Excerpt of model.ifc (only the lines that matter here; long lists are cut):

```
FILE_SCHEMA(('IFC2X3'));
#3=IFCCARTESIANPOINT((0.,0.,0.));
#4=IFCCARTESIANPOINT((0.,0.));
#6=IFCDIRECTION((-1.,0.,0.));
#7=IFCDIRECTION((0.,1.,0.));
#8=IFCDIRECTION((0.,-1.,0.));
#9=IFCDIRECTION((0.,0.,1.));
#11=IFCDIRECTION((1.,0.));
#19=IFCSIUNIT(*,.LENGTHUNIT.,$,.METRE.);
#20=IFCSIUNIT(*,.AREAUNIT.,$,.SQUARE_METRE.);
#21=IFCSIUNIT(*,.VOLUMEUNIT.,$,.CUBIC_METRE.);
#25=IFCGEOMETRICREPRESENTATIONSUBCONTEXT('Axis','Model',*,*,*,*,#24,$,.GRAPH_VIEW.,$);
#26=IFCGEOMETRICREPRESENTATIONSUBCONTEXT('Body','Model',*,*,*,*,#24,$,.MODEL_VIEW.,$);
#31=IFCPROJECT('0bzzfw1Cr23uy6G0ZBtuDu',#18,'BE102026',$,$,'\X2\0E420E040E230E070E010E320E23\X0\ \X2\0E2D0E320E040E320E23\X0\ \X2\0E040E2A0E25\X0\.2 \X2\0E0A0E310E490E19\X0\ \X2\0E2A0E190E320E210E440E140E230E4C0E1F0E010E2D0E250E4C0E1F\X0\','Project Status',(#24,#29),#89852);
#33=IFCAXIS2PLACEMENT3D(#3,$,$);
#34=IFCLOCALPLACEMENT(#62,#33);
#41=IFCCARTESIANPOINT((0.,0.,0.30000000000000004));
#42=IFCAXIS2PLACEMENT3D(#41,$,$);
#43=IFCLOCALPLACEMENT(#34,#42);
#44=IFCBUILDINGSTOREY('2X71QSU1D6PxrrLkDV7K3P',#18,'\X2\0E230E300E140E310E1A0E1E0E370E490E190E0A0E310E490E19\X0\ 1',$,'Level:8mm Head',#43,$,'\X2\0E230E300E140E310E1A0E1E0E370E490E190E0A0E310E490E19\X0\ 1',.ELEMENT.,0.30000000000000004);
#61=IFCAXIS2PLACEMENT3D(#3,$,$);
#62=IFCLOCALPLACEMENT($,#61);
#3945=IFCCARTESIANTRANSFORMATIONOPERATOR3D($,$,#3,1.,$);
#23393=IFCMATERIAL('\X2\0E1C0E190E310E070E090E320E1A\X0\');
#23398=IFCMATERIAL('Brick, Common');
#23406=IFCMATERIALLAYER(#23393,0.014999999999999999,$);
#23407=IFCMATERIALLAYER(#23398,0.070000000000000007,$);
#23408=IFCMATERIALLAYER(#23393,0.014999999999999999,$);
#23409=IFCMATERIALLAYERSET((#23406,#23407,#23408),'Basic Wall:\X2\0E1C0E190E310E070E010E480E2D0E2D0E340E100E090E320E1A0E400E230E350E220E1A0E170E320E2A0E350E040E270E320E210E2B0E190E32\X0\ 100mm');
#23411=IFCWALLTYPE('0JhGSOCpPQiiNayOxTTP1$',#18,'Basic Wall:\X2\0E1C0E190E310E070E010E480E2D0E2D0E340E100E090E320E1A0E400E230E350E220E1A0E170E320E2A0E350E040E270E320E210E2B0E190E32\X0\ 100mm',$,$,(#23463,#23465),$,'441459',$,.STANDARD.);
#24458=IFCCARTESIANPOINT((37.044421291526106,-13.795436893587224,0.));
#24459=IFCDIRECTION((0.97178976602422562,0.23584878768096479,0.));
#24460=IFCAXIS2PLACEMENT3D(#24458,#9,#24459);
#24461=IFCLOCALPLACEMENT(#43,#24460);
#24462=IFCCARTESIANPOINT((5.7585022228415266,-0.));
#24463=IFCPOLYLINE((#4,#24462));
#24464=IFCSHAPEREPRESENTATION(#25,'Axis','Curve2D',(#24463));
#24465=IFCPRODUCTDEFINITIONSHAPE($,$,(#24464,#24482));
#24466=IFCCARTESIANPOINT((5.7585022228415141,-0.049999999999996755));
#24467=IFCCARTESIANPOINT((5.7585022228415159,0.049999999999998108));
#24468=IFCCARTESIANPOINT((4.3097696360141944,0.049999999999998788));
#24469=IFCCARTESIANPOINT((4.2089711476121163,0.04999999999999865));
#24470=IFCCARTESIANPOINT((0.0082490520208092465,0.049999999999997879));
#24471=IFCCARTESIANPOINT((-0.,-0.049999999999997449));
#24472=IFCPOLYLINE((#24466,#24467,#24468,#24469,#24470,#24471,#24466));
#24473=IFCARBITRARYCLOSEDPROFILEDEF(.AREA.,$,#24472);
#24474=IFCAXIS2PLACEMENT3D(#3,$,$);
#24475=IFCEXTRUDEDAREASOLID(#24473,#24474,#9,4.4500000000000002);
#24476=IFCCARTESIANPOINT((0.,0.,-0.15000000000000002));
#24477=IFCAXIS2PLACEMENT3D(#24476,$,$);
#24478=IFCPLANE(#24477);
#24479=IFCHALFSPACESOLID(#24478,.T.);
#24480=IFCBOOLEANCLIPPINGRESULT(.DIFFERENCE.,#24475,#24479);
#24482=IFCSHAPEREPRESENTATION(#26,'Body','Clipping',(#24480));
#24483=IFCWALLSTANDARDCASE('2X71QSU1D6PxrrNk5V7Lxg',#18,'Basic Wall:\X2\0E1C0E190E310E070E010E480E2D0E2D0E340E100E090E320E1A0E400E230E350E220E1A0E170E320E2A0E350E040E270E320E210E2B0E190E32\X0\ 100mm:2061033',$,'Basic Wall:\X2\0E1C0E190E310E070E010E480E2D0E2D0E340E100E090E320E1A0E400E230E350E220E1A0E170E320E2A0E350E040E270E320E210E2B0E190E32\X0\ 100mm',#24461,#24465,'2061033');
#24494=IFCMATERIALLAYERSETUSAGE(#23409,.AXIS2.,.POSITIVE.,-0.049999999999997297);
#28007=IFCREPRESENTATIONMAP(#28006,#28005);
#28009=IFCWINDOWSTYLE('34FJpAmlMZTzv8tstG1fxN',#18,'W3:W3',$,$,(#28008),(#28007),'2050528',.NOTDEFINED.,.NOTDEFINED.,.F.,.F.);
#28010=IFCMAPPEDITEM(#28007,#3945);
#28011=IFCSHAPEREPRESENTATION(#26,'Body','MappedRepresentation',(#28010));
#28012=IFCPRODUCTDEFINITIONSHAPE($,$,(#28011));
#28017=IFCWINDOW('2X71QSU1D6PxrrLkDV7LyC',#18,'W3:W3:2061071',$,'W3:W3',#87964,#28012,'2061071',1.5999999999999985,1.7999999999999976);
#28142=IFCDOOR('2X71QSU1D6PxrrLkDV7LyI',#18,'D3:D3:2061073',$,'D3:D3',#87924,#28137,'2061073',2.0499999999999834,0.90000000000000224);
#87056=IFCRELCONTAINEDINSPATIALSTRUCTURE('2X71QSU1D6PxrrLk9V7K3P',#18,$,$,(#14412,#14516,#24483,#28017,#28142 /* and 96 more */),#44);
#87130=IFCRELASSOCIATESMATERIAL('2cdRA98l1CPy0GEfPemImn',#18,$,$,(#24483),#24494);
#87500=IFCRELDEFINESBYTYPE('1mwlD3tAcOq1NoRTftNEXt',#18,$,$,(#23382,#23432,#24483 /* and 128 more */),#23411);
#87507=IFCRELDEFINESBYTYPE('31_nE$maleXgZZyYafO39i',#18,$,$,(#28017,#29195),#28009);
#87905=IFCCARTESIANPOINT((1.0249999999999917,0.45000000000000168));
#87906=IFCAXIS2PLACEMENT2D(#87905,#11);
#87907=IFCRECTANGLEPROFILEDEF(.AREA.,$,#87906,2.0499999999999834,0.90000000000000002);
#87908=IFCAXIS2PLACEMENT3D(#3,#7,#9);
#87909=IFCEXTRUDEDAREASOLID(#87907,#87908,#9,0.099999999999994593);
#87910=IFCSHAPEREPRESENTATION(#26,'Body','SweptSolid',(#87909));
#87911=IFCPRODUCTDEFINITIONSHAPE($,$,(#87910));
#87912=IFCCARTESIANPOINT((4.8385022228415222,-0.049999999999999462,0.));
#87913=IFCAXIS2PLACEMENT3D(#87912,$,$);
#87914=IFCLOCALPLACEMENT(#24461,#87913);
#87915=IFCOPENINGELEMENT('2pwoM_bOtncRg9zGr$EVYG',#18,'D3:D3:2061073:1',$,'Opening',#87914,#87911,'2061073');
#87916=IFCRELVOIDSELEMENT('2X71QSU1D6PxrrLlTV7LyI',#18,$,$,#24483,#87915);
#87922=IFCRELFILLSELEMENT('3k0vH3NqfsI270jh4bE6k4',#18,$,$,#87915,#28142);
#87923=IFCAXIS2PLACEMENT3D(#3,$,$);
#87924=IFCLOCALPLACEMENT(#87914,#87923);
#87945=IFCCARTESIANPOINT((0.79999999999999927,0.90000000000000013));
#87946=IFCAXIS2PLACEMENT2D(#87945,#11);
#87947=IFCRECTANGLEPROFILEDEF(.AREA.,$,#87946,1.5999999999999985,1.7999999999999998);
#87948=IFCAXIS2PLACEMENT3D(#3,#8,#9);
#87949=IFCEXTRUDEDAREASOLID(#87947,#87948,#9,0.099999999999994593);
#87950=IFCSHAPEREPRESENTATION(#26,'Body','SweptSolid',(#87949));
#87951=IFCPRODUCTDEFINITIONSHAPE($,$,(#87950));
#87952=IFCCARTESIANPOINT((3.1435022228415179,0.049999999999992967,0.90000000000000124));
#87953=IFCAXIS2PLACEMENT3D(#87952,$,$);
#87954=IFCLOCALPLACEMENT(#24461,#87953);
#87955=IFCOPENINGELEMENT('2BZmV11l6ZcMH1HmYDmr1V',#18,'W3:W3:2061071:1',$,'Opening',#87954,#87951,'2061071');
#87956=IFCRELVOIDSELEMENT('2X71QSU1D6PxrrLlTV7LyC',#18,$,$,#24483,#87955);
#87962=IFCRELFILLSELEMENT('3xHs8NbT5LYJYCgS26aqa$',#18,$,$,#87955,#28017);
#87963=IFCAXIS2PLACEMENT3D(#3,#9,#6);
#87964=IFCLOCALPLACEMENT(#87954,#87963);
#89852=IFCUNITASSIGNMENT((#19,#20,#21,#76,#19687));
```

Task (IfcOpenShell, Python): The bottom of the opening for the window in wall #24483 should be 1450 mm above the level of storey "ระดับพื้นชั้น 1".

```python
import numpy as np
import ifcopenshell
import ifcopenshell.api.geometry
import ifcopenshell.geom
import ifcopenshell.util.element
import ifcopenshell.util.placement
import ifcopenshell.util.shape
import ifcopenshell.util.unit

model = ifcopenshell.open("model.ifc")
unit_scale = ifcopenshell.util.unit.calculate_unit_scale(model)

window = model.by_guid("2X71QSU1D6PxrrLkDV7LyC")
opening = window.FillsVoids[0].RelatingOpeningElement
storey = ifcopenshell.util.element.get_container(window, ifc_class="IfcBuildingStorey")
level = ifcopenshell.util.placement.get_local_placement(storey.ObjectPlacement)[2, 3]

# The opening's origin need not be at the sill, so measure its lowest point.
shape = ifcopenshell.geom.create_shape(ifcopenshell.geom.settings(), opening)
bottom = ifcopenshell.util.shape.get_shape_bottom_elevation(shape, shape.geometry) / unit_scale
dz = level + 1.45 / unit_scale - bottom

shift = np.array([0.0, 0.0, dz])
# The window is placed relative to its opening, so it follows when the opening moves.
matrix = ifcopenshell.util.placement.get_local_placement(opening.ObjectPlacement)
matrix[:3, 3] += shift
ifcopenshell.api.geometry.edit_object_placement(
    model, product=opening, matrix=matrix, is_si=False, should_transform_children=True
)

print(f"moved by {dz * unit_scale:+.3f} m")

model.write("model_edited.ifc")
```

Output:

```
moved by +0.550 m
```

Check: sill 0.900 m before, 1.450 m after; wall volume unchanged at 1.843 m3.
